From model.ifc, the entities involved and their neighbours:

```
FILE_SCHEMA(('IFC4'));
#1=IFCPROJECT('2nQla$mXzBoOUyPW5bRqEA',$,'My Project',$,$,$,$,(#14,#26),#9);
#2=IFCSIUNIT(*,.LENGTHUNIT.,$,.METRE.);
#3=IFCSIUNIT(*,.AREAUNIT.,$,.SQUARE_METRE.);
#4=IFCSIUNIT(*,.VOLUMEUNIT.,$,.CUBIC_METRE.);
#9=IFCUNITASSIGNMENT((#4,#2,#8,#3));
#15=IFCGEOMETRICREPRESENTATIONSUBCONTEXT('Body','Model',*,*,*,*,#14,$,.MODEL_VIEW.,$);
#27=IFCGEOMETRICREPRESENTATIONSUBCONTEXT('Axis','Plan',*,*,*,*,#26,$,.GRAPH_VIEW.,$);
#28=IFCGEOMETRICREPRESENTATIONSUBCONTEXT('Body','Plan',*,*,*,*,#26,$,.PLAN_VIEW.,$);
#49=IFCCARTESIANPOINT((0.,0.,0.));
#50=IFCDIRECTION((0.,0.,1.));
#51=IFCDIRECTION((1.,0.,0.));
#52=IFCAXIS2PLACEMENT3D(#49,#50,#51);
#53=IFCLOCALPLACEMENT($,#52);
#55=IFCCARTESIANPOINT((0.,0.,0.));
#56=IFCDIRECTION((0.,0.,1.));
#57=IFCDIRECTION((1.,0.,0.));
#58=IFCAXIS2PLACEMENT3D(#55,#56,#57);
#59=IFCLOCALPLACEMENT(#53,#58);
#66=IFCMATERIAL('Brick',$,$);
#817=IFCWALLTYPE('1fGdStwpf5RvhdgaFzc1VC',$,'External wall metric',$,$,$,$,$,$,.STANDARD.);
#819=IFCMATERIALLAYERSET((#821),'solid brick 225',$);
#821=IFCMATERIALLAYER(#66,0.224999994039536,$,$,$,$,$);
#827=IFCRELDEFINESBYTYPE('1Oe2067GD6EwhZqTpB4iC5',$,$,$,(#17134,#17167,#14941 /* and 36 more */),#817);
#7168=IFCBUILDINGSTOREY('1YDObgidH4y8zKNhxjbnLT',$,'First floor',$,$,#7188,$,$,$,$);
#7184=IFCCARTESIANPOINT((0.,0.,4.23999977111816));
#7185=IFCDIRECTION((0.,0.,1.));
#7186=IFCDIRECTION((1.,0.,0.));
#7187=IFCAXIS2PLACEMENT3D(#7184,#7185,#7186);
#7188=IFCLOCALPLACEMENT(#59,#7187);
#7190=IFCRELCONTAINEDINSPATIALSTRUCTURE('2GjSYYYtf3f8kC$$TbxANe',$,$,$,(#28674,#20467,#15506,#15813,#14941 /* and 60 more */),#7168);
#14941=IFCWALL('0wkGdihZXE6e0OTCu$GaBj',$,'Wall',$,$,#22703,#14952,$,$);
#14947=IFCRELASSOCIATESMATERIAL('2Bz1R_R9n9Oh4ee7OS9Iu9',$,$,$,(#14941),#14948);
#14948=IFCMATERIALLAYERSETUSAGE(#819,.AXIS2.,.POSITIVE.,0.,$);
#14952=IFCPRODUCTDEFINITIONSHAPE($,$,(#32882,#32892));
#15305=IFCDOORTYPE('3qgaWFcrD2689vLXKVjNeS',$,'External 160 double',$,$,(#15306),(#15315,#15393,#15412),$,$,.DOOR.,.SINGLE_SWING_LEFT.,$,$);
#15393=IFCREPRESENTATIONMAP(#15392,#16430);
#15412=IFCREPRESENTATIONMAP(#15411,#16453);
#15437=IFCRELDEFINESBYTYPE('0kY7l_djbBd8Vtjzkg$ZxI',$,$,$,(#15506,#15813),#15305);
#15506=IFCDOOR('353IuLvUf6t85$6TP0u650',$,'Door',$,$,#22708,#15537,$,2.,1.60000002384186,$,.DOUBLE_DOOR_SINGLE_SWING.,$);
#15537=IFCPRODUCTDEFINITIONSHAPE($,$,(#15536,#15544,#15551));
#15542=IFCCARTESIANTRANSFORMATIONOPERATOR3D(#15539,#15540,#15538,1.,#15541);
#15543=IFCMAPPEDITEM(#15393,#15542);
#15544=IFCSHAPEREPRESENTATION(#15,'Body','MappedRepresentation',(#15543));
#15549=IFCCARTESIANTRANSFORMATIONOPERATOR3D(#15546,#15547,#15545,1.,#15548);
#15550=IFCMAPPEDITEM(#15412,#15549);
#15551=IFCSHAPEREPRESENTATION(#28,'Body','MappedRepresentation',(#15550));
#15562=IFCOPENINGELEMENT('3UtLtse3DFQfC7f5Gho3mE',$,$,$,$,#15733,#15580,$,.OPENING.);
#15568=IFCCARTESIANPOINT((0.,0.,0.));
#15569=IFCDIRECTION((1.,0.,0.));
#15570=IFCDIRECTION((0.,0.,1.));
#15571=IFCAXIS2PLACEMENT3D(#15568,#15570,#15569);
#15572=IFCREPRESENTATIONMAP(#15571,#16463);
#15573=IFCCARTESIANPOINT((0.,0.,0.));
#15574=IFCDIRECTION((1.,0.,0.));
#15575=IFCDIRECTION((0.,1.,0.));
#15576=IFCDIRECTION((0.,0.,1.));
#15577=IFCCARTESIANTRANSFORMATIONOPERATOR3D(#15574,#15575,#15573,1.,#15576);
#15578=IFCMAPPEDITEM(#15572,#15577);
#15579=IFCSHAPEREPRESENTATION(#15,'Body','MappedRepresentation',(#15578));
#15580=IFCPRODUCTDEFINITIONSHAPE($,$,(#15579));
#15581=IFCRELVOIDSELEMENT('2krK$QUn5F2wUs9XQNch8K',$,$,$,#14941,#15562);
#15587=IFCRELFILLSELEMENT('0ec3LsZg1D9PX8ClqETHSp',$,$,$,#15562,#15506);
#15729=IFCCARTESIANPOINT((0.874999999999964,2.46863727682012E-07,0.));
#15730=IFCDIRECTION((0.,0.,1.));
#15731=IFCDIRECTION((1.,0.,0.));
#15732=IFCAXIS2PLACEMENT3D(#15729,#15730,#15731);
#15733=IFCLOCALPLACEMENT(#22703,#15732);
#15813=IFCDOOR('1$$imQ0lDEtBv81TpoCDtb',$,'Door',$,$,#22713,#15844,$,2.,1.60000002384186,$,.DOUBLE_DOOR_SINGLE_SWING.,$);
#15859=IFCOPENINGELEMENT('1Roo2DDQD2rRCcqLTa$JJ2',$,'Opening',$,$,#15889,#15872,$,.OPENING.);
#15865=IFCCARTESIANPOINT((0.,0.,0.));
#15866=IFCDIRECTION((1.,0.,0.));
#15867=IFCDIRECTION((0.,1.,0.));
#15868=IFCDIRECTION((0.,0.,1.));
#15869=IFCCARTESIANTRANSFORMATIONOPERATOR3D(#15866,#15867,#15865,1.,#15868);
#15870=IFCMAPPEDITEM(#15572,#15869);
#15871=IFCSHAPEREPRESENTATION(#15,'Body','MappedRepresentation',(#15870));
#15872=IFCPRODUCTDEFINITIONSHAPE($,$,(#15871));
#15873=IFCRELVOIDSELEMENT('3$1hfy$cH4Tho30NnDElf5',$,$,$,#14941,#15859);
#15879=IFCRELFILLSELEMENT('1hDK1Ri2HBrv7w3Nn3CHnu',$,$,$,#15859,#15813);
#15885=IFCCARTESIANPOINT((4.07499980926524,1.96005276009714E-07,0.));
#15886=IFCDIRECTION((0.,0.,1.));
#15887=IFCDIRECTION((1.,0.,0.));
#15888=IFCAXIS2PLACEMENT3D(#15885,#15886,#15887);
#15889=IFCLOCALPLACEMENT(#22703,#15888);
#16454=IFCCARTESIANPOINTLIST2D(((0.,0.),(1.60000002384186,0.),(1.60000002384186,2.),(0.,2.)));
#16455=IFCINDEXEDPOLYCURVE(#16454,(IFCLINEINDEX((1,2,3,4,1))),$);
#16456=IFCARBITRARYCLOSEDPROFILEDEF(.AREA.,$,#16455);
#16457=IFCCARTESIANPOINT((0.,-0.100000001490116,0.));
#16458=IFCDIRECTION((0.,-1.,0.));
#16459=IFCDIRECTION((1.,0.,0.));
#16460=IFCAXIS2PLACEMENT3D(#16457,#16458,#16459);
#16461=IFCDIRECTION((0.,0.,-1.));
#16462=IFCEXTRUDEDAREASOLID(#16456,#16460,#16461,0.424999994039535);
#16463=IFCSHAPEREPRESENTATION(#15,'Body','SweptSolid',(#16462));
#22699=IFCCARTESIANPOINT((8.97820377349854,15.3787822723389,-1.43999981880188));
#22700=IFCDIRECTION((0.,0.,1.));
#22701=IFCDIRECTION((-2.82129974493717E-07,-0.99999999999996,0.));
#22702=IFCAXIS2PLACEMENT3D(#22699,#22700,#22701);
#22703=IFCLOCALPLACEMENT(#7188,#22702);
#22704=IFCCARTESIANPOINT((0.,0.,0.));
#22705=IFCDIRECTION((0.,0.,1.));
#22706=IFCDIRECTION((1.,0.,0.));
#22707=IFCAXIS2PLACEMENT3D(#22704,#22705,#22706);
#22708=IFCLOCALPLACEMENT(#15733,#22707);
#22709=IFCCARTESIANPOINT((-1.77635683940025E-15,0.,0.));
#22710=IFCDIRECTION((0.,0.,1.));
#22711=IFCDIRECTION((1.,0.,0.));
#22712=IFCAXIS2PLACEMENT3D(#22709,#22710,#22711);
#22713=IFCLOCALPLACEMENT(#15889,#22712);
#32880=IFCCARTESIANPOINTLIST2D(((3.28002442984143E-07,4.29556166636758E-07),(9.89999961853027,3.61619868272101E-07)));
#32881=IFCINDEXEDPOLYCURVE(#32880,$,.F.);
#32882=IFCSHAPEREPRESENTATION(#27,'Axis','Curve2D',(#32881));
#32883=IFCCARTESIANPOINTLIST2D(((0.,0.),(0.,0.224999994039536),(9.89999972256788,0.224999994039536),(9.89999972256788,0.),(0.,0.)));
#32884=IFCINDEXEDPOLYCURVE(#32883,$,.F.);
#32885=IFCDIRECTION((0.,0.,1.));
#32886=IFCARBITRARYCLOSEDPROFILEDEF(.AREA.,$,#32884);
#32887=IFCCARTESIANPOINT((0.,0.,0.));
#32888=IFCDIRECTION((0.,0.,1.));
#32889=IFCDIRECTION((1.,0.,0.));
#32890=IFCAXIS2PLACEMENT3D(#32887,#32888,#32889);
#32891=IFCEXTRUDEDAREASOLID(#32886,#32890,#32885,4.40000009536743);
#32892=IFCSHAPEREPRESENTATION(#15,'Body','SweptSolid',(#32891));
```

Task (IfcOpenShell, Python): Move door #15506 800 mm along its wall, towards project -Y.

```python
import ifcopenshell
import ifcopenshell.api.geometry
import ifcopenshell.util.placement
import ifcopenshell.util.unit

model = ifcopenshell.open("model.ifc")
unit_scale = ifcopenshell.util.unit.calculate_unit_scale(model)

door = model.by_guid("353IuLvUf6t85$6TP0u650")
opening = door.FillsVoids[0].RelatingOpeningElement
wall = opening.VoidsElements[0].RelatingBuildingElement

wall_matrix = ifcopenshell.util.placement.get_local_placement(wall.ObjectPlacement)
shift = wall_matrix[:3, 0] * 0.8 / unit_scale
before = ifcopenshell.util.placement.get_local_placement(door.ObjectPlacement)[:3, 3].copy()

# The door is placed relative to its opening, so it follows when the opening moves.
matrix = ifcopenshell.util.placement.get_local_placement(opening.ObjectPlacement)
matrix[:3, 3] += shift
ifcopenshell.api.geometry.edit_object_placement(
    model, product=opening, matrix=matrix, is_si=False, should_transform_children=True
)

after = ifcopenshell.util.placement.get_local_placement(door.ObjectPlacement)[:3, 3]
print("door moved by", (after - before).round(3) + 0.0)

model.write("model_edited.ifc")
```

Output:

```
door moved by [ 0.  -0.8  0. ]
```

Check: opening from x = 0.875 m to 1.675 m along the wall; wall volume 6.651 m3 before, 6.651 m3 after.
